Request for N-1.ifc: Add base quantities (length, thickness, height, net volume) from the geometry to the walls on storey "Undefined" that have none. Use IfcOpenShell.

First a look at what the model holds.

```python
import ifcopenshell
import ifcopenshell.util.element
import ifcopenshell.util.unit

model = ifcopenshell.open("N-1.ifc")
print(model.schema)
for unit_type in ("LENGTHUNIT", "AREAUNIT", "VOLUMEUNIT"):
    print(unit_type, ifcopenshell.util.unit.calculate_unit_scale(model, unit_type))
storey = next(s for s in model.by_type("IfcBuildingStorey") if s.Name == "Undefined")
walls = [e for e in ifcopenshell.util.element.get_decomposition(storey) if e.is_a("IfcWall")]
for e in sorted(walls, key=lambda e: e.id()):
    print(e.id(), e.is_a(), e.Name, list(ifcopenshell.util.element.get_psets(e, qtos_only=True)), sep=" | ")
```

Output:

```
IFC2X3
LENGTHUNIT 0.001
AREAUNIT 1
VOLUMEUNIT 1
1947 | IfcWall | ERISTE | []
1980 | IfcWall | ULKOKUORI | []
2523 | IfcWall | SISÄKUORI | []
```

```python
import ifcopenshell
import ifcopenshell.api.pset
import ifcopenshell.geom
import ifcopenshell.util.element
import ifcopenshell.util.shape
import ifcopenshell.util.unit

model = ifcopenshell.open("N-1.ifc")
unit_scale = ifcopenshell.util.unit.calculate_unit_scale(model)
volume_scale = ifcopenshell.util.unit.calculate_unit_scale(model, "VOLUMEUNIT")
settings = ifcopenshell.geom.settings()

storey = next(s for s in model.by_type("IfcBuildingStorey") if s.Name == "Undefined")
walls = [e for e in ifcopenshell.util.element.get_decomposition(storey) if e.is_a("IfcWall")]

for e in sorted(walls, key=lambda e: e.id()):
    if ifcopenshell.util.element.get_psets(e, qtos_only=True, should_inherit=False):
        continue
    # Geometry comes back in metres, in the element's own axes.
    shape = ifcopenshell.geom.create_shape(settings, e)
    values = {
        "Length": ifcopenshell.util.shape.get_x(shape.geometry) / unit_scale,
        "Width": ifcopenshell.util.shape.get_y(shape.geometry) / unit_scale,
        "Height": ifcopenshell.util.shape.get_z(shape.geometry) / unit_scale,
        "NetVolume": ifcopenshell.util.shape.get_volume(shape.geometry) / volume_scale,
    }
    qto = ifcopenshell.api.pset.add_qto(model, product=e, name="BaseQuantities")
    ifcopenshell.api.pset.edit_qto(model, qto=qto, properties=values)
    print(e.id(), {k: round(v, 3) for k, v in values.items()})

model.write("N-1_edited.ifc")
```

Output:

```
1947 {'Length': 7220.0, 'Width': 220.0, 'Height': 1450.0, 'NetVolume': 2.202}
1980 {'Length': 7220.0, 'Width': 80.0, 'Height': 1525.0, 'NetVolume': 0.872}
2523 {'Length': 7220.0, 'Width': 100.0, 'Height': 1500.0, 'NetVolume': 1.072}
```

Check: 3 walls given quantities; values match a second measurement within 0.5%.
